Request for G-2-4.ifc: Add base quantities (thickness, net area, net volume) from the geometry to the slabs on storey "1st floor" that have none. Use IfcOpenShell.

First a look at what the model holds.

```python
import ifcopenshell
import ifcopenshell.util.element
import ifcopenshell.util.unit

model = ifcopenshell.open("G-2-4.ifc")
print(model.schema)
for unit_type in ("LENGTHUNIT", "AREAUNIT", "VOLUMEUNIT"):
    print(unit_type, ifcopenshell.util.unit.calculate_unit_scale(model, unit_type))
storey = next(s for s in model.by_type("IfcBuildingStorey") if s.Name == "1st floor")
slabs = [e for e in ifcopenshell.util.element.get_decomposition(storey) if e.is_a("IfcSlab")]
for e in sorted(slabs, key=lambda e: e.id()):
    print(e.id(), e.is_a(), e.Name, list(ifcopenshell.util.element.get_psets(e, qtos_only=True)), sep=" | ")
```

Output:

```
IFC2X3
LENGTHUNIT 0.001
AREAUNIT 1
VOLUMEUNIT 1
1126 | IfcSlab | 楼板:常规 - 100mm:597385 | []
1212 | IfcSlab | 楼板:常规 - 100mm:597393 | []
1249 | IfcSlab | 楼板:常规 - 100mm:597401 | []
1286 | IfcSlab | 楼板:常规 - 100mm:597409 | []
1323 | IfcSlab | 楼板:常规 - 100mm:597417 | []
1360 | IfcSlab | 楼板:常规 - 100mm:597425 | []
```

```python
import ifcopenshell
import ifcopenshell.api.pset
import ifcopenshell.geom
import ifcopenshell.util.element
import ifcopenshell.util.shape
import ifcopenshell.util.unit

model = ifcopenshell.open("G-2-4.ifc")
unit_scale = ifcopenshell.util.unit.calculate_unit_scale(model)
area_scale = ifcopenshell.util.unit.calculate_unit_scale(model, "AREAUNIT")
volume_scale = ifcopenshell.util.unit.calculate_unit_scale(model, "VOLUMEUNIT")
settings = ifcopenshell.geom.settings()

storey = next(s for s in model.by_type("IfcBuildingStorey") if s.Name == "1st floor")
slabs = [e for e in ifcopenshell.util.element.get_decomposition(storey) if e.is_a("IfcSlab")]

for e in sorted(slabs, key=lambda e: e.id()):
    if ifcopenshell.util.element.get_psets(e, qtos_only=True, should_inherit=False):
        continue
    # Geometry comes back in metres, in the element's own axes.
    shape = ifcopenshell.geom.create_shape(settings, e)
    values = {
        "Width": ifcopenshell.util.shape.get_z(shape.geometry) / unit_scale,
        "NetArea": ifcopenshell.util.shape.get_footprint_area(shape.geometry) / area_scale,
        "NetVolume": ifcopenshell.util.shape.get_volume(shape.geometry) / volume_scale,
    }
    qto = ifcopenshell.api.pset.add_qto(model, product=e, name="BaseQuantities")
    ifcopenshell.api.pset.edit_qto(model, qto=qto, properties=values)
    print(e.id(), {k: round(v, 3) for k, v in values.items()})

model.write("G-2-4-out.ifc")
```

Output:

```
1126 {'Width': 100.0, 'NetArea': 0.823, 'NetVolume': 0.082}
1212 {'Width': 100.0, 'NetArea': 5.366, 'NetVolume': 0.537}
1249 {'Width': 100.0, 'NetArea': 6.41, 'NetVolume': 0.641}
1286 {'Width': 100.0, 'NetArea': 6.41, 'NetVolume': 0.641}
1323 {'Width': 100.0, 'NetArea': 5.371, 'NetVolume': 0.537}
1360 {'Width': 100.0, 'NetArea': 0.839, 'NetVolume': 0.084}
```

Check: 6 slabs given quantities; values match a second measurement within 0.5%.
